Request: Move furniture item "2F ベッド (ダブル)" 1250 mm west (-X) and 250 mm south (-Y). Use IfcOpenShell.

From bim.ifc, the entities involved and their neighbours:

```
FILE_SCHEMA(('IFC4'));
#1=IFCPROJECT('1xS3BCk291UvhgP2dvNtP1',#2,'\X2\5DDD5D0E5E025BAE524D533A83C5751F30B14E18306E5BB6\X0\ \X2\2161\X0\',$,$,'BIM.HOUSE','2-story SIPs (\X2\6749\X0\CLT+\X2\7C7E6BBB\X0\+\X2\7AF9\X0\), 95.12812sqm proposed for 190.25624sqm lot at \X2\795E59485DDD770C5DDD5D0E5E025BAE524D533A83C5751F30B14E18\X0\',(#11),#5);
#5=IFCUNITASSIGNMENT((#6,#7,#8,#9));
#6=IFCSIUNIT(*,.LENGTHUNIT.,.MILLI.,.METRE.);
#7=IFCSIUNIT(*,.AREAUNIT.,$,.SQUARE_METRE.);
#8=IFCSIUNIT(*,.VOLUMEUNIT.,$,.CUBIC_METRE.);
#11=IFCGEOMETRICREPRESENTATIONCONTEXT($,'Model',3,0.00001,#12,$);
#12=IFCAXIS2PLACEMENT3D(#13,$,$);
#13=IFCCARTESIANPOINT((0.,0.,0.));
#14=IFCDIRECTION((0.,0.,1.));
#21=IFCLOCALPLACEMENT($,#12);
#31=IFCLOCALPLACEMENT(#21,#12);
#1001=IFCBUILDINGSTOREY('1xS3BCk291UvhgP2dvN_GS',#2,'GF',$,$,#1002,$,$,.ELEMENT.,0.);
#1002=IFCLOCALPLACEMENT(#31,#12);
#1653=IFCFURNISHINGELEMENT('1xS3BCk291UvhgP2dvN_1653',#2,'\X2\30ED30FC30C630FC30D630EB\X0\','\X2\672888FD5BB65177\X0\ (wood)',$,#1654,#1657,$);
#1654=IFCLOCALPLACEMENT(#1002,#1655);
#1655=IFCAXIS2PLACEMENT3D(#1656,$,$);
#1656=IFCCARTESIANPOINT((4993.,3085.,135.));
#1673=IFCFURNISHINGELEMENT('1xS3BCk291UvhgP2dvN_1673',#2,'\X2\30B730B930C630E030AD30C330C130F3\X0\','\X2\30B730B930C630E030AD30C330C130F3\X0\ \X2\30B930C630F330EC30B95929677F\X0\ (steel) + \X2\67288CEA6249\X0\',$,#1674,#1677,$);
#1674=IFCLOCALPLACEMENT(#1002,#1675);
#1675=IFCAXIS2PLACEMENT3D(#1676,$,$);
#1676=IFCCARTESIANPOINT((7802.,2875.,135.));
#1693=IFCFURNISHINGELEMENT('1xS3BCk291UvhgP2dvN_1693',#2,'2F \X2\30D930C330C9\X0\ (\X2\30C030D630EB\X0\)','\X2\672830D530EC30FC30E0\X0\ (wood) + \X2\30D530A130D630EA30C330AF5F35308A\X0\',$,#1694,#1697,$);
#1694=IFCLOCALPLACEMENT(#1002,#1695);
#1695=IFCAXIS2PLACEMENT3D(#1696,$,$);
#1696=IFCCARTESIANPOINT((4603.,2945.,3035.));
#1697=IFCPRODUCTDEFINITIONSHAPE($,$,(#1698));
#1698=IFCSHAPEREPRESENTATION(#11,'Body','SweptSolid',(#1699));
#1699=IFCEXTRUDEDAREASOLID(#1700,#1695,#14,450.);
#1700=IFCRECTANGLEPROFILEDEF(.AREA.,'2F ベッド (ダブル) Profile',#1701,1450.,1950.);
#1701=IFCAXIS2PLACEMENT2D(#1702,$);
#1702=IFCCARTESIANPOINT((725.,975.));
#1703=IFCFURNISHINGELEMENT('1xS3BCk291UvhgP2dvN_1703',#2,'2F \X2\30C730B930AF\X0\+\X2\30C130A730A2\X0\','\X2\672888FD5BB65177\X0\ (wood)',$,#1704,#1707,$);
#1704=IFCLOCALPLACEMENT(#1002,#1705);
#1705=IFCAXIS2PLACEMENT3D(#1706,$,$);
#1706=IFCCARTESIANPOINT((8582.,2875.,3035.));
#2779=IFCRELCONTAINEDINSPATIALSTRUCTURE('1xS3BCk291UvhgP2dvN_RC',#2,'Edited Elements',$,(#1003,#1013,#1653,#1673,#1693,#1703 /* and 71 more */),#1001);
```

```python
import ifcopenshell
import ifcopenshell.api.geometry
import ifcopenshell.util.placement

model = ifcopenshell.open("bim.ifc")

item = model.by_guid("1xS3BCk291UvhgP2dvN_1693")
matrix = ifcopenshell.util.placement.get_local_placement(item.ObjectPlacement)
matrix[0, 3] -= 1250.0
matrix[1, 3] -= 250.0
ifcopenshell.api.geometry.edit_object_placement(model, product=item, matrix=matrix, is_si=False)

print(ifcopenshell.util.placement.get_local_placement(item.ObjectPlacement).round(3) + 0.0)

model.write("bim_updated.ifc")
```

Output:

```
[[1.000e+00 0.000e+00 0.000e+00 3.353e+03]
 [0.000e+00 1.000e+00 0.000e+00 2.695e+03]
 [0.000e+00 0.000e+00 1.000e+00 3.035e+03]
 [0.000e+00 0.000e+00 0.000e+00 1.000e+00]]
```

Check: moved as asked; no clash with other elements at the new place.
